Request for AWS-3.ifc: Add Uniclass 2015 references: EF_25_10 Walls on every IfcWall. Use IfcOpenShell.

First a look at what the model holds.

```python
import ifcopenshell

model = ifcopenshell.open("AWS-3.ifc")
print(model.schema)
print("classifications:", [c.Name for c in model.by_type("IfcClassification")])
for ifc_class in ("IfcDoor", "IfcRoof", "IfcStair", "IfcWall", "IfcWindow"):
    print(ifc_class, len(model.by_type(ifc_class)))
```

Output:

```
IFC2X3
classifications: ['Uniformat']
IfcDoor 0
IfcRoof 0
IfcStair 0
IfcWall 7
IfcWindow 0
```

```python
import ifcopenshell
import ifcopenshell.api.classification

model = ifcopenshell.open("AWS-3.ifc")

# IFC2X3 requires Source and Edition and has no link from the project to the system.
system = model.create_entity("IfcClassification", Source="NBS", Edition="2015", Name="Uniclass 2015")

codes = {
    "IfcWall": ("EF_25_10", "Walls"),
}
for ifc_class, (code, name) in codes.items():
    products = model.by_type(ifc_class)
    ifcopenshell.api.classification.add_reference(
        model, products=products, classification=system, identification=code, name=name
    )
    print(code, len(products))

model.write("AWS-3_rev.ifc")
```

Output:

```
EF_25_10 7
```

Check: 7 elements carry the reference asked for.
